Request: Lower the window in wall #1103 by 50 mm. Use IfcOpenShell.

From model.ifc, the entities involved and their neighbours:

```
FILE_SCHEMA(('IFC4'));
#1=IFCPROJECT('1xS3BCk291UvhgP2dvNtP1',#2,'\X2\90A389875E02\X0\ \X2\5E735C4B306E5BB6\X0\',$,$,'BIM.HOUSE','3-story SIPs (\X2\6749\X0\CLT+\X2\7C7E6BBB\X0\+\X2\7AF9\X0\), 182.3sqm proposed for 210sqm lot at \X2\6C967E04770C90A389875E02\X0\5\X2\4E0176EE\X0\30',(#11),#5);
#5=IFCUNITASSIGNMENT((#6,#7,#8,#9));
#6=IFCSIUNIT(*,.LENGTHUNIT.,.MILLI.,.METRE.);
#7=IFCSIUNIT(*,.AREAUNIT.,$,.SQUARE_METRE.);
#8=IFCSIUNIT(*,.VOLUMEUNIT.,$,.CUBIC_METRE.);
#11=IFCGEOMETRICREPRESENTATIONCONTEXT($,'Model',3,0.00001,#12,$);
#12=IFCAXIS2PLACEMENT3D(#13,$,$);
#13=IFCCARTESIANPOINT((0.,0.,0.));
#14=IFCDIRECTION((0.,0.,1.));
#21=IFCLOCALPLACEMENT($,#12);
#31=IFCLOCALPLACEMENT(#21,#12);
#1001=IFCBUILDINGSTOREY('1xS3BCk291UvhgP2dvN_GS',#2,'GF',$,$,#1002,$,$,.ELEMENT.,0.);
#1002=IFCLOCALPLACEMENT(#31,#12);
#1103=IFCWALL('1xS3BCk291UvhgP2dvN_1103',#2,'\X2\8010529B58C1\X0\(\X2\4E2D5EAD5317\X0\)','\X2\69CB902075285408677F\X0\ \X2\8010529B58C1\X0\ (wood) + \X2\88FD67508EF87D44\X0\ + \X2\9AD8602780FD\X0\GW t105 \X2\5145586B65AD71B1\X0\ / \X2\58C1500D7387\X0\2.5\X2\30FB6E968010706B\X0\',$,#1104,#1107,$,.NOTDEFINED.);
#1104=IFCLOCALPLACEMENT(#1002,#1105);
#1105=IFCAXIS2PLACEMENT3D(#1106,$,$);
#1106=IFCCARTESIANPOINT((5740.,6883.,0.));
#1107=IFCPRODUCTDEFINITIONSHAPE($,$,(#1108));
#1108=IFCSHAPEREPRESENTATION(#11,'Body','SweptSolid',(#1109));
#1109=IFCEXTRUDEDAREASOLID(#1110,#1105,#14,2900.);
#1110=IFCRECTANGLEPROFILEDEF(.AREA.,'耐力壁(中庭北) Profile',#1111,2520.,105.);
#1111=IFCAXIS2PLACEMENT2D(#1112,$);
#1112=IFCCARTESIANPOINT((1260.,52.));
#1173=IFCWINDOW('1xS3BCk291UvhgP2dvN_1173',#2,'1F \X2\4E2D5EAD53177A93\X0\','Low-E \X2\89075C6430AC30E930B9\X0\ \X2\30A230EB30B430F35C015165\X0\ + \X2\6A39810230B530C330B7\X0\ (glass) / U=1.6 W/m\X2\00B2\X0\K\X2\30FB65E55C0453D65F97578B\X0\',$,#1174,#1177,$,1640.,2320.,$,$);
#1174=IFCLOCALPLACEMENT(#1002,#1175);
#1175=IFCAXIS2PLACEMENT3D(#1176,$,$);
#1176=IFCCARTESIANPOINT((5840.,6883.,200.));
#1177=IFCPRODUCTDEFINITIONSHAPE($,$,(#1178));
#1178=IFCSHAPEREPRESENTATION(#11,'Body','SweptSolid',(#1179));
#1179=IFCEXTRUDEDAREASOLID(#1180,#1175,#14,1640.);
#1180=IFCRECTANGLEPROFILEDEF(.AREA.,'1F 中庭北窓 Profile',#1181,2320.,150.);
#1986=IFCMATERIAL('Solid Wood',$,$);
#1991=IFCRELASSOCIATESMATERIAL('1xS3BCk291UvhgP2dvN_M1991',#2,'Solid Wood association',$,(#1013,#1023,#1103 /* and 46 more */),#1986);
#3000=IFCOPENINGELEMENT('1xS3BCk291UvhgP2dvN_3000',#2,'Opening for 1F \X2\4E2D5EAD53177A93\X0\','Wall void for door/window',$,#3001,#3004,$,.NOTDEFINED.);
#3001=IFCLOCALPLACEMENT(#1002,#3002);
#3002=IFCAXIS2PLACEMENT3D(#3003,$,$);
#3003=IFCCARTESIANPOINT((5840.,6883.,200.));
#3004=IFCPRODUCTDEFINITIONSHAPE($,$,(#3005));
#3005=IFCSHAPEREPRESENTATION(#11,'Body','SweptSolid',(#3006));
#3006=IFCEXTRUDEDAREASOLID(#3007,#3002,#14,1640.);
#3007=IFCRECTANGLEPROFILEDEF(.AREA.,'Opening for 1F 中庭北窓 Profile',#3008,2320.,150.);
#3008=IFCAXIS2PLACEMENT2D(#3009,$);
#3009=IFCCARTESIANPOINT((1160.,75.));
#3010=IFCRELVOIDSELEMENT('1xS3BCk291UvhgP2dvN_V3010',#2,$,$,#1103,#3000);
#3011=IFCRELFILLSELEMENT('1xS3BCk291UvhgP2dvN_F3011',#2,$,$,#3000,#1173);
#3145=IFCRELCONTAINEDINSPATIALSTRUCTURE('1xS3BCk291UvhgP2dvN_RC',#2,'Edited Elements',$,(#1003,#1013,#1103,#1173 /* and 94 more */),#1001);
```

```python
import numpy as np
import ifcopenshell
import ifcopenshell.api.geometry
import ifcopenshell.util.placement
import ifcopenshell.util.unit

model = ifcopenshell.open("model.ifc")
unit_scale = ifcopenshell.util.unit.calculate_unit_scale(model)

window = model.by_guid("1xS3BCk291UvhgP2dvN_1173")
opening = window.FillsVoids[0].RelatingOpeningElement
dz = -50.0

shift = np.array([0.0, 0.0, dz])
# The window is not placed relative to its opening, so move both.
for product in (opening, window):
    matrix = ifcopenshell.util.placement.get_local_placement(product.ObjectPlacement)
    matrix[:3, 3] += shift
    ifcopenshell.api.geometry.edit_object_placement(model, product=product, matrix=matrix, is_si=False)

print(f"moved by {dz * unit_scale:+.3f} m")

model.write("model_updated.ifc")
```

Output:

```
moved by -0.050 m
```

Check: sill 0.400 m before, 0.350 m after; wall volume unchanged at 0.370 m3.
